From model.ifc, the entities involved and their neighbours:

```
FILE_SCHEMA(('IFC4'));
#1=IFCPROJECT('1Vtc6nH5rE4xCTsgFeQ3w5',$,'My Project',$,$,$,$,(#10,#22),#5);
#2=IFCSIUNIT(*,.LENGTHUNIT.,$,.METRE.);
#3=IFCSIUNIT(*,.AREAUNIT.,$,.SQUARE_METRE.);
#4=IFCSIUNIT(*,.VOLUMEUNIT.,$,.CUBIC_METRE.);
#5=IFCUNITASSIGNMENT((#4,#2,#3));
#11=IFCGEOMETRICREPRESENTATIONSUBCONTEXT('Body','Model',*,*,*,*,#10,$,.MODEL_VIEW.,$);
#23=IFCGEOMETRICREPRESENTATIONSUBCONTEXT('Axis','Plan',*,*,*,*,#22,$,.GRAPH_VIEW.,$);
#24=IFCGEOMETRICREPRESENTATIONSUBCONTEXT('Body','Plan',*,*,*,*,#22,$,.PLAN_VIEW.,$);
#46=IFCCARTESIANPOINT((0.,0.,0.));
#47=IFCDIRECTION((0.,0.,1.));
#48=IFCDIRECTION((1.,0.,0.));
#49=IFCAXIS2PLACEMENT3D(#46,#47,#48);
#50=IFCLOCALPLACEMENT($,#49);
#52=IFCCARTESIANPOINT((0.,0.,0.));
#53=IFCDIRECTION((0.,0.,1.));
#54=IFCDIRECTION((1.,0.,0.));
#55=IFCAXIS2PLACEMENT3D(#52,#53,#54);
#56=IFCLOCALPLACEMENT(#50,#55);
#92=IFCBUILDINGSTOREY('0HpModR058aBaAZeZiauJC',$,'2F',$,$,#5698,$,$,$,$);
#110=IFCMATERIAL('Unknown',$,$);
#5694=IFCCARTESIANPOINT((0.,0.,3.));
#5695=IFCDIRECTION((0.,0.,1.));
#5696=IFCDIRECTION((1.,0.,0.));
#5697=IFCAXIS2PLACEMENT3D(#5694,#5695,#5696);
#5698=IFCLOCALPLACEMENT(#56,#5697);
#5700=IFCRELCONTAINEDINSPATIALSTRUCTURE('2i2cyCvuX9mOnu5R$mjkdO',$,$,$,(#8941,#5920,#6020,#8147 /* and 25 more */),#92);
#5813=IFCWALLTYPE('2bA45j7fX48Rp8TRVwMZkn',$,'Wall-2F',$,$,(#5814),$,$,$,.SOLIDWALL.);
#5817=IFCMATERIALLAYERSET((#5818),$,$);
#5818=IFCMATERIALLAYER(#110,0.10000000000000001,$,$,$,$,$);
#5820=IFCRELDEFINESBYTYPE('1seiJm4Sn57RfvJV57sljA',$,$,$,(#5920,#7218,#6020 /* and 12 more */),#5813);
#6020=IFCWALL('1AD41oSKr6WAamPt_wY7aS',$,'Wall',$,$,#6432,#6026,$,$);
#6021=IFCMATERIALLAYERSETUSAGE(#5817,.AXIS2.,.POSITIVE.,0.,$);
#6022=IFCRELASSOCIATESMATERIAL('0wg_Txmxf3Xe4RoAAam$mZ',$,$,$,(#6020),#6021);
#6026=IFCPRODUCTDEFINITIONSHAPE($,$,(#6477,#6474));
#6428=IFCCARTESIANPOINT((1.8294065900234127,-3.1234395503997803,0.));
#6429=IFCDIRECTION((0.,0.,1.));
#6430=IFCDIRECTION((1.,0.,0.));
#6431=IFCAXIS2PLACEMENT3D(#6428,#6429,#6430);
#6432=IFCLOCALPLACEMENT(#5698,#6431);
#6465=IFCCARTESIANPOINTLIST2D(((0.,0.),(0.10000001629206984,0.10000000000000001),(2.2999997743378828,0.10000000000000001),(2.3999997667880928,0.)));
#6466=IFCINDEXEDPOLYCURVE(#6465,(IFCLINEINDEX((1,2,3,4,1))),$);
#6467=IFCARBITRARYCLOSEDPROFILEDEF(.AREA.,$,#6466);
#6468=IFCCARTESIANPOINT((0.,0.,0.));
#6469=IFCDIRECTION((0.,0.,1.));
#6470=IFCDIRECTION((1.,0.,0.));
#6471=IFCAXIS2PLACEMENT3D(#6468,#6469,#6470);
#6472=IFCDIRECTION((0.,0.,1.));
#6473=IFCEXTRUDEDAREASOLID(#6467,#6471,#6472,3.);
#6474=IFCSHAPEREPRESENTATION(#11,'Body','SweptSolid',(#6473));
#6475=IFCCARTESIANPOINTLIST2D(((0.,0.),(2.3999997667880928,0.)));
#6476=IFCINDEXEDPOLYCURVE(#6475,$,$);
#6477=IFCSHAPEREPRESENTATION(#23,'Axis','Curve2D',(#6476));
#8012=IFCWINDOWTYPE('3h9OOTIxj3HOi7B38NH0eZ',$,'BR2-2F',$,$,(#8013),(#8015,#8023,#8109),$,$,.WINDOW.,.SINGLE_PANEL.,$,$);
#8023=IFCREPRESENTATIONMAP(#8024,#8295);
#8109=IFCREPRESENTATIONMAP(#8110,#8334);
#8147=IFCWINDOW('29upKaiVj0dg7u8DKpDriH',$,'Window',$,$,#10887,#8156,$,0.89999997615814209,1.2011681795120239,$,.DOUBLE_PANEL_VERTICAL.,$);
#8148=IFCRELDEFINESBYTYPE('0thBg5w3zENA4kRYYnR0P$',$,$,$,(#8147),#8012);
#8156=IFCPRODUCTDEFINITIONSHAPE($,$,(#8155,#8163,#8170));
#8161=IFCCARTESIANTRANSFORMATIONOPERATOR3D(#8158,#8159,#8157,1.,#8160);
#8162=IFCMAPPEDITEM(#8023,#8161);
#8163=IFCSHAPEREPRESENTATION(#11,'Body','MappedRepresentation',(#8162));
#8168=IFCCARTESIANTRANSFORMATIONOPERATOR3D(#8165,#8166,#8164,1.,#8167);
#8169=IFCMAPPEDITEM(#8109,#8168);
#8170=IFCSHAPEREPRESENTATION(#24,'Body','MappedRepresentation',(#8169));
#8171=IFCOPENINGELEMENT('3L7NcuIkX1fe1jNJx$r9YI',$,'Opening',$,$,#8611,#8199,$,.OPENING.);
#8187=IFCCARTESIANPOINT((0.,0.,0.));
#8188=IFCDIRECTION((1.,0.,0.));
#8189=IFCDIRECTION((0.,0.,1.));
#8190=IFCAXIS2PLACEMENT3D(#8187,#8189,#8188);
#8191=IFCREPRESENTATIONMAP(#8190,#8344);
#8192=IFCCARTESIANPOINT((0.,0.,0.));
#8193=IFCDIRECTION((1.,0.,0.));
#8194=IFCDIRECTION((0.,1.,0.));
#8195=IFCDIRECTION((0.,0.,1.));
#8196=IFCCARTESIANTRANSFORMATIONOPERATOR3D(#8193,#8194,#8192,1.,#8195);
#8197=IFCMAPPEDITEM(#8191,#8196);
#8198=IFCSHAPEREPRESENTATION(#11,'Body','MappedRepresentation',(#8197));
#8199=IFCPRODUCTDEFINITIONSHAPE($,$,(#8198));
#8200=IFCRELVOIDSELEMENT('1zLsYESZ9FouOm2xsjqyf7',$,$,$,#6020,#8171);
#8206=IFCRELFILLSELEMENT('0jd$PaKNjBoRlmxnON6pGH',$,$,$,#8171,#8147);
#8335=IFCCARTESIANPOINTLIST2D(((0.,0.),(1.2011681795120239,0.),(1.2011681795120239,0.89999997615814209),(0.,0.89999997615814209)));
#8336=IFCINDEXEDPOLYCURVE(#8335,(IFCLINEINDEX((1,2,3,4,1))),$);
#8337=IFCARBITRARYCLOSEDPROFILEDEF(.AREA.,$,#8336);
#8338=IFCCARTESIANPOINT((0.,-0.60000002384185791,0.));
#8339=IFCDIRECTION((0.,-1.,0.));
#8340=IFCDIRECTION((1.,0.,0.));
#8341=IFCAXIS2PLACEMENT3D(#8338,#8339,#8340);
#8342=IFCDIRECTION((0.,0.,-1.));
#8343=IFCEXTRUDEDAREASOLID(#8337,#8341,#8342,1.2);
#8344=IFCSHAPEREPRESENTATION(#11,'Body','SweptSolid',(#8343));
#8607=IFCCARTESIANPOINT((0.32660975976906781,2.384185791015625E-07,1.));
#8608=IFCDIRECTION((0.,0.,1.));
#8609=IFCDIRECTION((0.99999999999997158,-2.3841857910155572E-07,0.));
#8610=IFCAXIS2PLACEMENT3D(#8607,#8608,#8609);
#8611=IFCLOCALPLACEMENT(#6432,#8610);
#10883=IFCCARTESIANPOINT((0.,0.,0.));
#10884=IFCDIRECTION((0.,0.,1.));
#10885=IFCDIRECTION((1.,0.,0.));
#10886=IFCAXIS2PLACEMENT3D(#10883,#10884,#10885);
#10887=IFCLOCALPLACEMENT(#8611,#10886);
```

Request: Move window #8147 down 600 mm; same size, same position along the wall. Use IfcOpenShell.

```python
import numpy as np
import ifcopenshell
import ifcopenshell.api.geometry
import ifcopenshell.util.placement
import ifcopenshell.util.unit

model = ifcopenshell.open("model.ifc")
unit_scale = ifcopenshell.util.unit.calculate_unit_scale(model)

window = model.by_id(8147)
opening = window.FillsVoids[0].RelatingOpeningElement
dz = -0.6 / unit_scale

shift = np.array([0.0, 0.0, dz])
# The window is placed relative to its opening, so it follows when the opening moves.
matrix = ifcopenshell.util.placement.get_local_placement(opening.ObjectPlacement)
matrix[:3, 3] += shift
ifcopenshell.api.geometry.edit_object_placement(
    model, product=opening, matrix=matrix, is_si=False, should_transform_children=True
)

print(f"moved by {dz * unit_scale:+.3f} m")

model.write("model_rev.ifc")
```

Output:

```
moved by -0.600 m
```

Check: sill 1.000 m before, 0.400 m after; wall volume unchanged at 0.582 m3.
